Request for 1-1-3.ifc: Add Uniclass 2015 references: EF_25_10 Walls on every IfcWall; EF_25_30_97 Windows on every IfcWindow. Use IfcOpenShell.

First a look at what the model holds.

```python
import ifcopenshell

model = ifcopenshell.open("1-1-3.ifc")
print(model.schema)
print("classifications:", [c.Name for c in model.by_type("IfcClassification")])
for ifc_class in ("IfcDoor", "IfcRoof", "IfcStair", "IfcWall", "IfcWindow"):
    print(ifc_class, len(model.by_type(ifc_class)))
```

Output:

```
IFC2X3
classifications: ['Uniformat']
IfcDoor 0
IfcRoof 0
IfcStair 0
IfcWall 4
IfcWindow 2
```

```python
import ifcopenshell
import ifcopenshell.api.classification

model = ifcopenshell.open("1-1-3.ifc")

# IFC2X3 requires Source and Edition and has no link from the project to the system.
system = model.create_entity("IfcClassification", Source="NBS", Edition="2015", Name="Uniclass 2015")

codes = {
    "IfcWall": ("EF_25_10", "Walls"),
    "IfcWindow": ("EF_25_30_97", "Windows"),
}
for ifc_class, (code, name) in codes.items():
    products = model.by_type(ifc_class)
    ifcopenshell.api.classification.add_reference(
        model, products=products, classification=system, identification=code, name=name
    )
    print(code, len(products))

model.write("1-1-3_edited.ifc")
```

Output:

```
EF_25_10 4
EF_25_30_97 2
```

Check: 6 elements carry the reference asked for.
